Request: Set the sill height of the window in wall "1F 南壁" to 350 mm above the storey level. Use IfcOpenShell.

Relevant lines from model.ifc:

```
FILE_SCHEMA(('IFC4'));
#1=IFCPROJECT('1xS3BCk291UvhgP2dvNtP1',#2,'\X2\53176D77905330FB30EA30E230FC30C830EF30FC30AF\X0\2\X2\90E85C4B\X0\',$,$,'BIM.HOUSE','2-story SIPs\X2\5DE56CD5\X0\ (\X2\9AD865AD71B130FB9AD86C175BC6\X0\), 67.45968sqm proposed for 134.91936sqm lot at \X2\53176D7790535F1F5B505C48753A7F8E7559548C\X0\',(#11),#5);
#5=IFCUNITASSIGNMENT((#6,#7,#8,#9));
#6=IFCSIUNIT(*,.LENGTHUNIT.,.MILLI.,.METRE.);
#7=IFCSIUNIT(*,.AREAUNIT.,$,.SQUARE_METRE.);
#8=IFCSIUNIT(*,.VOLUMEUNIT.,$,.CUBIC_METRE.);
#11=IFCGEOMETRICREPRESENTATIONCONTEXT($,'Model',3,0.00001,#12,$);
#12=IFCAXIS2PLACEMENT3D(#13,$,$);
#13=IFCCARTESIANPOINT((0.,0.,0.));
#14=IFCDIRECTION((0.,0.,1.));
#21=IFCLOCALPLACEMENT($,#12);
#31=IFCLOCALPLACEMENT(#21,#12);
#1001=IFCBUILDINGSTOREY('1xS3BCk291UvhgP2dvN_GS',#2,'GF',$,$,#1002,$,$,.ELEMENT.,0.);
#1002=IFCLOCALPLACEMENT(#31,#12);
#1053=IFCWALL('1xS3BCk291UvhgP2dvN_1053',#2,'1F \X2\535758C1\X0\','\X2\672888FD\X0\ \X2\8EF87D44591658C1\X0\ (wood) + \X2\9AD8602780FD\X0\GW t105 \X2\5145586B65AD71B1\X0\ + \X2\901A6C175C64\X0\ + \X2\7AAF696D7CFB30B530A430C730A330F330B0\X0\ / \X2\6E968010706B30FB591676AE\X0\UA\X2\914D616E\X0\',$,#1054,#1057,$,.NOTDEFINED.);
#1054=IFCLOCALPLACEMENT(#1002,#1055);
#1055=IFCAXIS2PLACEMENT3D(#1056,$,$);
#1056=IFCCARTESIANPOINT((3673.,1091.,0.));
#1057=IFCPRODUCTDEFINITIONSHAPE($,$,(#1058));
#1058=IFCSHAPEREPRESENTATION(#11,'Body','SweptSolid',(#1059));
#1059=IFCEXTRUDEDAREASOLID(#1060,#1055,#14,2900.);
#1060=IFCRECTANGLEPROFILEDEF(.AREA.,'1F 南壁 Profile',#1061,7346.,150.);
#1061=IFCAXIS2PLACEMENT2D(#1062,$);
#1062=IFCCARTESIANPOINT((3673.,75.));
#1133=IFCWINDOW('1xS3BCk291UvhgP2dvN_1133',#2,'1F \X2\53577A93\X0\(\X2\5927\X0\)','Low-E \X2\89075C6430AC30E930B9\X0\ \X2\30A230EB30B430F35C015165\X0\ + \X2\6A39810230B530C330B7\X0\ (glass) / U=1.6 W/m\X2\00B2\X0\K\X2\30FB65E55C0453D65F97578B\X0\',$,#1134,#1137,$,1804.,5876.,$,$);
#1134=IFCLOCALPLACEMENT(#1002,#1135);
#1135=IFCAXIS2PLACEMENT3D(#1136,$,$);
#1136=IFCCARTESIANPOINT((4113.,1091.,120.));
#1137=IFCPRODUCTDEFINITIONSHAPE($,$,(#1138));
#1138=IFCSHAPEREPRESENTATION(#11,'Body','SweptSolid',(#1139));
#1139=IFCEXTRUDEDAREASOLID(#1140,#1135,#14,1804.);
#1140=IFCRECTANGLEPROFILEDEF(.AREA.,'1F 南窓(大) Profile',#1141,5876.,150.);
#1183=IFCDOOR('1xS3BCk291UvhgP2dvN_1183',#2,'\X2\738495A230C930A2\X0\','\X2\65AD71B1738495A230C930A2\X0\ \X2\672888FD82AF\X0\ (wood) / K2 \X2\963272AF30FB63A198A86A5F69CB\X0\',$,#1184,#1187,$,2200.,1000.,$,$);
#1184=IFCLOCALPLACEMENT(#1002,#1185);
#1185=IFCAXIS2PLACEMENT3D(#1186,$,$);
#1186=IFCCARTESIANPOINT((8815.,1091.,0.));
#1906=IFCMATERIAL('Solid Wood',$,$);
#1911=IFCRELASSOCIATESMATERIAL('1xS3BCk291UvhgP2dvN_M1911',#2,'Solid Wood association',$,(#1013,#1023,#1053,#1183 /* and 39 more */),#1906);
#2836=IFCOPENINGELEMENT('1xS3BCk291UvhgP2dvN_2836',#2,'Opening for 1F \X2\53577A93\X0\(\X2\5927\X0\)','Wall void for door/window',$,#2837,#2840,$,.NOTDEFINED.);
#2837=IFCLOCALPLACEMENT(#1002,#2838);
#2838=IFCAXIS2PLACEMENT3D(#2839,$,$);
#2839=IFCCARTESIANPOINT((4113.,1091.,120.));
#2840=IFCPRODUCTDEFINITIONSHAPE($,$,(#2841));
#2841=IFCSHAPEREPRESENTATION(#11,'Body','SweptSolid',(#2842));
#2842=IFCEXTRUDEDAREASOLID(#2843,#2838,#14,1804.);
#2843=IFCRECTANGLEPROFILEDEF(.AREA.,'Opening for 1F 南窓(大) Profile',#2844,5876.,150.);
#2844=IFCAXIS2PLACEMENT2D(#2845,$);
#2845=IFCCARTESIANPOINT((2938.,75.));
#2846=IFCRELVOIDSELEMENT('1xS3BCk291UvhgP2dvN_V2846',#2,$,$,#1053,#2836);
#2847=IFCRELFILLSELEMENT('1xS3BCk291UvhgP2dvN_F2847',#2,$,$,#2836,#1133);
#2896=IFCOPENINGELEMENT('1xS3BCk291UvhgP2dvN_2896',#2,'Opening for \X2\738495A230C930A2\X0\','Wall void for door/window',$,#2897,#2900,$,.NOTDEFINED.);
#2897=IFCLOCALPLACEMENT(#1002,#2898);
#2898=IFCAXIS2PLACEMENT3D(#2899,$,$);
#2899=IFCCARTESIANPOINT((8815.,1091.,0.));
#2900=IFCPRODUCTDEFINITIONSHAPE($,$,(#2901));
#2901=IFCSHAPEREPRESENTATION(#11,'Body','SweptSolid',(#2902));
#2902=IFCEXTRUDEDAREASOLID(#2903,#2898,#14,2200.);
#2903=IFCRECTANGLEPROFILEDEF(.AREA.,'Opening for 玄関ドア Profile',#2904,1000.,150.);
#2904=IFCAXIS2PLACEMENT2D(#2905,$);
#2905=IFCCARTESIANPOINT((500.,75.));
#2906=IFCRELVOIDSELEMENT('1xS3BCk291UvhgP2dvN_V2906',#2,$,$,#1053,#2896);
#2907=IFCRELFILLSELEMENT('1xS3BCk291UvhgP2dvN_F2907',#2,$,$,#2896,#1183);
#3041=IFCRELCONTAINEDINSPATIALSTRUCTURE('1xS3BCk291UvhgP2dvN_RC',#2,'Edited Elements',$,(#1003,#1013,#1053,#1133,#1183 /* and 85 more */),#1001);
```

```python
import numpy as np
import ifcopenshell
import ifcopenshell.api.geometry
import ifcopenshell.geom
import ifcopenshell.util.element
import ifcopenshell.util.placement
import ifcopenshell.util.shape
import ifcopenshell.util.unit

model = ifcopenshell.open("model.ifc")
unit_scale = ifcopenshell.util.unit.calculate_unit_scale(model)

window = model.by_guid("1xS3BCk291UvhgP2dvN_1133")
opening = window.FillsVoids[0].RelatingOpeningElement
storey = ifcopenshell.util.element.get_container(window, ifc_class="IfcBuildingStorey")
level = ifcopenshell.util.placement.get_local_placement(storey.ObjectPlacement)[2, 3]

# The opening's origin need not be at the sill, so measure its lowest point.
shape = ifcopenshell.geom.create_shape(ifcopenshell.geom.settings(), opening)
bottom = ifcopenshell.util.shape.get_shape_bottom_elevation(shape, shape.geometry) / unit_scale
dz = level + 0.35 / unit_scale - bottom

shift = np.array([0.0, 0.0, dz])
# The window is not placed relative to its opening, so move both.
for product in (opening, window):
    matrix = ifcopenshell.util.placement.get_local_placement(product.ObjectPlacement)
    matrix[:3, 3] += shift
    ifcopenshell.api.geometry.edit_object_placement(model, product=product, matrix=matrix, is_si=False)

print(f"moved by {dz * unit_scale:+.3f} m")

model.write("model_rev.ifc")
```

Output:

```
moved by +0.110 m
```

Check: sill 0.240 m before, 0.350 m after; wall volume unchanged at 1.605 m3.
